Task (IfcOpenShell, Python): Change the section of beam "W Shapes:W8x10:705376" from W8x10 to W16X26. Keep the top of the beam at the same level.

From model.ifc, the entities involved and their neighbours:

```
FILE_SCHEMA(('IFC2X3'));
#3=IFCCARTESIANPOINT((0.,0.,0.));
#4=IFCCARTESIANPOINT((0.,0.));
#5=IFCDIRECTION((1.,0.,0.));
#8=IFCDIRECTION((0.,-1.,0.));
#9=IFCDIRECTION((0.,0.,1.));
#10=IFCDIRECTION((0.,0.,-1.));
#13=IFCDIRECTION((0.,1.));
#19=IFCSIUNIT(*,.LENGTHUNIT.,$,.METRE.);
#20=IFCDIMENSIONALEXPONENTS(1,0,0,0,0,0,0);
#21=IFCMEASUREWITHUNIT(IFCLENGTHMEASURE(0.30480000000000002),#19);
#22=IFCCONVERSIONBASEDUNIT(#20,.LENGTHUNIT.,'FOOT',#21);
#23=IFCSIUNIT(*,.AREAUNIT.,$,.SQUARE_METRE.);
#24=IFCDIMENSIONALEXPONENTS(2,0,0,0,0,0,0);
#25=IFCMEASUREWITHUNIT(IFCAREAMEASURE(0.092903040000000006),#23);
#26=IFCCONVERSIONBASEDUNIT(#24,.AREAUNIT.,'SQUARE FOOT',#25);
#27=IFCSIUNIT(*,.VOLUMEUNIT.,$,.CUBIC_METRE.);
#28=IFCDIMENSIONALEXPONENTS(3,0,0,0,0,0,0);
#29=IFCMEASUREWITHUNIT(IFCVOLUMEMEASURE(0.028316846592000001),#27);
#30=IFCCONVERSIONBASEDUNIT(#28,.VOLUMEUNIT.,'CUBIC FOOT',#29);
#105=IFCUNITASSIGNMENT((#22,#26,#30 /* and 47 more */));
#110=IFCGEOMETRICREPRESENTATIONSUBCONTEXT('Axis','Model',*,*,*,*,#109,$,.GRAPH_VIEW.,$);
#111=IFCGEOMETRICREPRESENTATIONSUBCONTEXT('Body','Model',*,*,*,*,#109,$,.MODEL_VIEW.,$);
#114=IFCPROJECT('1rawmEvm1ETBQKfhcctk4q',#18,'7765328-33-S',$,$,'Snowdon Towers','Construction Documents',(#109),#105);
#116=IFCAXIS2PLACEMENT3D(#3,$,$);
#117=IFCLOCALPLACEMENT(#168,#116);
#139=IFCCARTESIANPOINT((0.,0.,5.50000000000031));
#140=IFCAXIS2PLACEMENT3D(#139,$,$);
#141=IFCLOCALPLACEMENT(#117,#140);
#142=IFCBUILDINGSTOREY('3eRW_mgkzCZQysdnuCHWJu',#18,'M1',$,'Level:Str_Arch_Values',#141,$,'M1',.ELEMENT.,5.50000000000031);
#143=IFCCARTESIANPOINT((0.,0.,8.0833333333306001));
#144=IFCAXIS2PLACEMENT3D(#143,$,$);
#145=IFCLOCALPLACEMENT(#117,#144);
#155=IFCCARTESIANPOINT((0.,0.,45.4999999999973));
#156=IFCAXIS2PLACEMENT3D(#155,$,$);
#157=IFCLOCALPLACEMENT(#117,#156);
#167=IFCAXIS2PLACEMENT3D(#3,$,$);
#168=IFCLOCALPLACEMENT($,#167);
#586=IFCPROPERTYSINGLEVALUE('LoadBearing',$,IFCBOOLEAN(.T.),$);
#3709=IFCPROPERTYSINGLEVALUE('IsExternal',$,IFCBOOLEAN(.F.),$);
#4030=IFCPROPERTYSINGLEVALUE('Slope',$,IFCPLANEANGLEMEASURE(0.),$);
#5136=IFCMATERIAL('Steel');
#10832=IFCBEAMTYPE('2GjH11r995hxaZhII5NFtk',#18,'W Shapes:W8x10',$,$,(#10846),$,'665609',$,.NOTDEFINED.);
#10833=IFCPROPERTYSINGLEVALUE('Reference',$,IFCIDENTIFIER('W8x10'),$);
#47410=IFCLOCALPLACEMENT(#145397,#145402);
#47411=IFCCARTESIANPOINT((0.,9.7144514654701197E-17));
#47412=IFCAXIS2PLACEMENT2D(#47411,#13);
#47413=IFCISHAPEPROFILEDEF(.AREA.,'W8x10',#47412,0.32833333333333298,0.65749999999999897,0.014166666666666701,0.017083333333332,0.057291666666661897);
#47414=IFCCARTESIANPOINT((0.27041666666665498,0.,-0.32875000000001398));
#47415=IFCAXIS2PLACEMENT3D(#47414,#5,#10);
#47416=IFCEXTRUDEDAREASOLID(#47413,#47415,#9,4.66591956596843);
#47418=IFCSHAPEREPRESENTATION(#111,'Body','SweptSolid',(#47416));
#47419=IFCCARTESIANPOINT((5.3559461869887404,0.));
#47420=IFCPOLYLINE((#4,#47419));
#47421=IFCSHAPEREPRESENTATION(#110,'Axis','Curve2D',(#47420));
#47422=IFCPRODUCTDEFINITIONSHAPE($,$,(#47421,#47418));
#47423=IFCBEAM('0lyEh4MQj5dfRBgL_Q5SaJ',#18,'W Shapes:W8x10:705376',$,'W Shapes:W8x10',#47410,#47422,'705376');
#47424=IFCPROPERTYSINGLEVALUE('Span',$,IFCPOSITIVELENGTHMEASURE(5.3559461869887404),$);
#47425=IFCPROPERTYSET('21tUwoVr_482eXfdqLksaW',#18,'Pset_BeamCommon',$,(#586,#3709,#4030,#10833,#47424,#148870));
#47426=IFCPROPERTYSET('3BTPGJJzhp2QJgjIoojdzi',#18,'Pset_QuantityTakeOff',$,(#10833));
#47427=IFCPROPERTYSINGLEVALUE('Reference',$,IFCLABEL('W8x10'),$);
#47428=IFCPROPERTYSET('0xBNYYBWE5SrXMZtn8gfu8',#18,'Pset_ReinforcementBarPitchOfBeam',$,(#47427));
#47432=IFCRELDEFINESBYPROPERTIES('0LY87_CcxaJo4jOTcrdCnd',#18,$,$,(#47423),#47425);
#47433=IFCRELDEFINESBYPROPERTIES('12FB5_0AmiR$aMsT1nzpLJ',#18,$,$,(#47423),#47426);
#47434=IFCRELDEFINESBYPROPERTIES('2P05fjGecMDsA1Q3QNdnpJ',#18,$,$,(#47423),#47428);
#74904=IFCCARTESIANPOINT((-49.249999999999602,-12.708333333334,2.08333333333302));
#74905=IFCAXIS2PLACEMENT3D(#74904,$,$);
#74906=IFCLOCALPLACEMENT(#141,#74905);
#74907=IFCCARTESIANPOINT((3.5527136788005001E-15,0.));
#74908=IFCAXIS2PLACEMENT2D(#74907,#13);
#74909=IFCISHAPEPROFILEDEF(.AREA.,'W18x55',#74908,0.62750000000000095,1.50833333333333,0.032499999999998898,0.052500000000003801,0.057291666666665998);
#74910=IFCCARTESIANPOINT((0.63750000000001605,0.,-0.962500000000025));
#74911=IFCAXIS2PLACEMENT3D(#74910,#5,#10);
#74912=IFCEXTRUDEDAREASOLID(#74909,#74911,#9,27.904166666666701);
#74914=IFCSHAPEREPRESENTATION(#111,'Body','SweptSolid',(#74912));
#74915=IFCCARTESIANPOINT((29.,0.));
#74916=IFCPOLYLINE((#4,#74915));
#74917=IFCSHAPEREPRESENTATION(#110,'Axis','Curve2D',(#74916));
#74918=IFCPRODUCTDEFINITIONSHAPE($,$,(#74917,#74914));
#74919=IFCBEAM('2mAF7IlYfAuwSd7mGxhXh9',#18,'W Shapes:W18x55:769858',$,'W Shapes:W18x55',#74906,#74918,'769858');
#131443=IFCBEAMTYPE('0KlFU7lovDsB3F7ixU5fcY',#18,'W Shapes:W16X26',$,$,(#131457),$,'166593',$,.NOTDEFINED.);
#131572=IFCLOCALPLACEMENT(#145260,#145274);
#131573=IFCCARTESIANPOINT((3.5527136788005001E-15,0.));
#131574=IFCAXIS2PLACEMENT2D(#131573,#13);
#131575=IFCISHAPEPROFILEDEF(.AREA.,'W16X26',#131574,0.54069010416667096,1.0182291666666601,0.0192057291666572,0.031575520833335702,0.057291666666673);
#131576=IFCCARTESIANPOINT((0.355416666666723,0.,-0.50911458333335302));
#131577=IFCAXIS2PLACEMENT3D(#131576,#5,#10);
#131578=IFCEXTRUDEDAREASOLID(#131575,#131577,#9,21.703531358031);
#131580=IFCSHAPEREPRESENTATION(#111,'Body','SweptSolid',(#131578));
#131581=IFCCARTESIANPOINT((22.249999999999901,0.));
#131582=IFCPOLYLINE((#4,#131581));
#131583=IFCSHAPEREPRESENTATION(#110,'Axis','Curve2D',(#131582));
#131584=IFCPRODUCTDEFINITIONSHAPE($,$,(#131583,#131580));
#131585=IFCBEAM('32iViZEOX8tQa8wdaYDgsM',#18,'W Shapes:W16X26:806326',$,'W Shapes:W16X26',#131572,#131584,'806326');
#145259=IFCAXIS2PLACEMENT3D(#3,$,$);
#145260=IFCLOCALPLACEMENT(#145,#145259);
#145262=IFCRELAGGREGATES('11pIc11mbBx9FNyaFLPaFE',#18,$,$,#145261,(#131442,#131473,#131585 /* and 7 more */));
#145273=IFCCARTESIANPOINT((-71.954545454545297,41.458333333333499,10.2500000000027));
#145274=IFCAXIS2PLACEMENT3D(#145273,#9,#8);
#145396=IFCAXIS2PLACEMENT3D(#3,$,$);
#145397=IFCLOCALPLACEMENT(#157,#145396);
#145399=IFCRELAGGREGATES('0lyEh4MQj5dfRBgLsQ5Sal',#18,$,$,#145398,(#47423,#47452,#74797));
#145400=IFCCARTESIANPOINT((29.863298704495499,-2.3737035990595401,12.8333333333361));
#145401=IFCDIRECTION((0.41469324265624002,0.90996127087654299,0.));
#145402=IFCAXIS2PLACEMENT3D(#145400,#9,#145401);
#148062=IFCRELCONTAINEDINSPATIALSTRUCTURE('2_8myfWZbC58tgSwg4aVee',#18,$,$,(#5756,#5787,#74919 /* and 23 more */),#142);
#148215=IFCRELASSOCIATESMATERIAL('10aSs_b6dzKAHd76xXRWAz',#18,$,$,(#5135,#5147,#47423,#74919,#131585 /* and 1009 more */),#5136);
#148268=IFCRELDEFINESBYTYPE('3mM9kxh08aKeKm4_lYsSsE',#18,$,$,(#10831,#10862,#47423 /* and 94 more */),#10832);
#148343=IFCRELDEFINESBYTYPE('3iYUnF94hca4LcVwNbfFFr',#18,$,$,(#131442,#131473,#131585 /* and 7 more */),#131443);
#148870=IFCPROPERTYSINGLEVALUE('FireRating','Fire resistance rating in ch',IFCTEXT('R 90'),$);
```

```python
import ifcopenshell
import ifcopenshell.api.pset
import ifcopenshell.api.type
import ifcopenshell.util.element
import ifcopenshell.util.representation

model = ifcopenshell.open("model.ifc")

member = model.by_guid("0lyEh4MQj5dfRBgL_Q5SaJ")
source = next(p for p in model.by_type("IfcIShapeProfileDef") if p.ProfileName == "W16X26")

body = ifcopenshell.util.representation.get_representation(member, "Model", "Body")
solid = body.Items[0]
old_profile = solid.SweptArea

# Copy the section's sizes but keep this member's own profile position.
profile = ifcopenshell.util.element.copy(model, source)
# Profiles are centred, so shift by half the change in depth to hold the top.
shift = (old_profile.OverallDepth - profile.OverallDepth) / 2
x, y = old_profile.Position.Location.Coordinates
up = (-1.0, 0.0)  # upwards, in the solid's own plane
location = model.createIfcCartesianPoint((x + up[0] * shift, y + up[1] * shift))
profile.Position = model.createIfcAxis2Placement2D(location, old_profile.Position.RefDirection)
solid.SweptArea = profile
if not model.get_total_inverses(old_profile):
    ifcopenshell.util.element.remove_deep2(model, old_profile)

new_type = model.by_id(131443)
ifcopenshell.api.type.assign_type(
    model, related_objects=[member], relating_type=new_type, should_map_representations=False
)
member.Name = member.Name.replace("W8x10", "W16X26")
member.ObjectType = "W Shapes:W16X26"
pset = model.by_id(ifcopenshell.util.element.get_pset(member, "Pset_BeamCommon", should_inherit=False)["id"])
ifcopenshell.api.pset.edit_pset(model, pset=pset, properties={"Reference": "W16X26"})
pset = model.by_id(ifcopenshell.util.element.get_pset(member, "Pset_QuantityTakeOff", should_inherit=False)["id"])
ifcopenshell.api.pset.edit_pset(model, pset=pset, properties={"Reference": "W16X26"})
pset = model.by_id(ifcopenshell.util.element.get_pset(member, "Pset_ReinforcementBarPitchOfBeam", should_inherit=False)["id"])
ifcopenshell.api.pset.edit_pset(model, pset=pset, properties={"Reference": "W16X26"})

print(solid.SweptArea)

model.write("model-out.ifc")
```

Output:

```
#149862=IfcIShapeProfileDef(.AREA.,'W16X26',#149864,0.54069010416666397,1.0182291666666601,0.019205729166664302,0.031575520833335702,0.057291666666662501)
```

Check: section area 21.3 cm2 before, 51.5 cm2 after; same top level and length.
